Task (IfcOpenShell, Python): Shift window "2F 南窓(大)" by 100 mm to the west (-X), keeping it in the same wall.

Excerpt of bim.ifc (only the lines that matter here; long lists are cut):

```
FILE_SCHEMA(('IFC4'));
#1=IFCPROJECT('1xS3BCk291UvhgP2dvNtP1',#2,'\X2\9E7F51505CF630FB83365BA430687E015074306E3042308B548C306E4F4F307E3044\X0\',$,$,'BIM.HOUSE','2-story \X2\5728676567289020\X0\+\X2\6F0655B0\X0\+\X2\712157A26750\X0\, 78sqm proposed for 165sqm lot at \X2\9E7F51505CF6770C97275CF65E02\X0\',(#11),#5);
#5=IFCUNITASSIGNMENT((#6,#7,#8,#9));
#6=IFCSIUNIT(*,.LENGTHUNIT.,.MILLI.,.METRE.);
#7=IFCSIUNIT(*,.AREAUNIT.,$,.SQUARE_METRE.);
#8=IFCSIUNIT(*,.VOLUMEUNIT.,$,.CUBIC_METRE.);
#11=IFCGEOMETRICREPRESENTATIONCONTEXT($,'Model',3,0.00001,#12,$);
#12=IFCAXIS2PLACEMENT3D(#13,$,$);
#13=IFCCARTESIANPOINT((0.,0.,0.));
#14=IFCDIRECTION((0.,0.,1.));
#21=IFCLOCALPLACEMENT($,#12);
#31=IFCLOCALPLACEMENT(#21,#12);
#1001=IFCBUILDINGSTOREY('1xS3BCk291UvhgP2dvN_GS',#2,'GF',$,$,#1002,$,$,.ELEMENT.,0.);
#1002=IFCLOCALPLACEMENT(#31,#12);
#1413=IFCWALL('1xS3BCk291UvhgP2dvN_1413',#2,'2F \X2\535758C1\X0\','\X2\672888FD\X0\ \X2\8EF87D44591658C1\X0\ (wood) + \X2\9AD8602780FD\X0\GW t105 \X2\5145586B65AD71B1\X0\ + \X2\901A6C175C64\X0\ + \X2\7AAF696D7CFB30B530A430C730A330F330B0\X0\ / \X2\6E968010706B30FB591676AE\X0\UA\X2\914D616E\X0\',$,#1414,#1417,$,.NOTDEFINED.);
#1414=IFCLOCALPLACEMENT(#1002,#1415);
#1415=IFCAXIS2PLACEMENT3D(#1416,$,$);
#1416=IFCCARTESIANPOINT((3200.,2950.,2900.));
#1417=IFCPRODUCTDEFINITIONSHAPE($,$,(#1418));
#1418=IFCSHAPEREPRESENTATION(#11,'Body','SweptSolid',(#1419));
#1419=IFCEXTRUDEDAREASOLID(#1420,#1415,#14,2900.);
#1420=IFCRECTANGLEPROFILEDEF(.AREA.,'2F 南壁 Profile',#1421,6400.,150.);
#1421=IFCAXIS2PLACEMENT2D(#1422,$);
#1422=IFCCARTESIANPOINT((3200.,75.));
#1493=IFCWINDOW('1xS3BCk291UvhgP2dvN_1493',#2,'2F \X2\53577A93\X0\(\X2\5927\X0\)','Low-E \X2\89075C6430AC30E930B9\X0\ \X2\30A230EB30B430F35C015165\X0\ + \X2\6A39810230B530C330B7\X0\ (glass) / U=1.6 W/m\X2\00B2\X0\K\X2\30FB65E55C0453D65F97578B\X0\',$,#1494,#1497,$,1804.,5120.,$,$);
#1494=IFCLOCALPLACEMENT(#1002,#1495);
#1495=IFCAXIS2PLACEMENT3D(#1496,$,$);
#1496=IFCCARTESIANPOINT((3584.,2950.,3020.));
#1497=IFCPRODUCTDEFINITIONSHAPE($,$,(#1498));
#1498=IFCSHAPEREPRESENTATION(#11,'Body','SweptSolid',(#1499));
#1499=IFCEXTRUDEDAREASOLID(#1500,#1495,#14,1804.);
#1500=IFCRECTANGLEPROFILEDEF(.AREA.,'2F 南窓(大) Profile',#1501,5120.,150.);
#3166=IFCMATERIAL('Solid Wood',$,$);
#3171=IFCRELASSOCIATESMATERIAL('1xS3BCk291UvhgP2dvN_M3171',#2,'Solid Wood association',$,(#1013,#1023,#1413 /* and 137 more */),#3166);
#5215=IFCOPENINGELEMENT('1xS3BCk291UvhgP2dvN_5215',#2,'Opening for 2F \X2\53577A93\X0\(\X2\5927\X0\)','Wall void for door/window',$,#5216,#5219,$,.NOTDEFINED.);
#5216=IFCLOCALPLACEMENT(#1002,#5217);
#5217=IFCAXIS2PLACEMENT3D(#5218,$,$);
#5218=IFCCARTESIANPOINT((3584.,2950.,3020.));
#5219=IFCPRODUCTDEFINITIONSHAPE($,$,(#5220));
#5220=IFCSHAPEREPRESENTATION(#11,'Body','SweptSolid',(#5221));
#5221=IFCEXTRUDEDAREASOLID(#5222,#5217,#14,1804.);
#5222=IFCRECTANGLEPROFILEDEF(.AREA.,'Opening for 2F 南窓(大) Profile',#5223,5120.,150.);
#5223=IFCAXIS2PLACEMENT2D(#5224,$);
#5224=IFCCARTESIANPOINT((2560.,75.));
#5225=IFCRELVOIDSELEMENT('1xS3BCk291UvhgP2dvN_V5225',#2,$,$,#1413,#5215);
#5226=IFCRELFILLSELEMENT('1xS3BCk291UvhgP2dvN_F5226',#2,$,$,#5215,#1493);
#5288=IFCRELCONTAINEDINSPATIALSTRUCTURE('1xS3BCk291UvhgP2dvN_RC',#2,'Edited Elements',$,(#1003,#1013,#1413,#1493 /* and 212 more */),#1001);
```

```python
import ifcopenshell
import ifcopenshell.api.geometry
import ifcopenshell.util.placement
import ifcopenshell.util.unit

model = ifcopenshell.open("bim.ifc")
unit_scale = ifcopenshell.util.unit.calculate_unit_scale(model)

window = model.by_guid("1xS3BCk291UvhgP2dvN_1493")
opening = window.FillsVoids[0].RelatingOpeningElement
wall = opening.VoidsElements[0].RelatingBuildingElement

wall_matrix = ifcopenshell.util.placement.get_local_placement(wall.ObjectPlacement)
shift = wall_matrix[:3, 0] * -0.1 / unit_scale
before = ifcopenshell.util.placement.get_local_placement(window.ObjectPlacement)[:3, 3].copy()

# The window is not placed relative to its opening, so move both.
for product in (opening, window):
    matrix = ifcopenshell.util.placement.get_local_placement(product.ObjectPlacement)
    matrix[:3, 3] += shift
    ifcopenshell.api.geometry.edit_object_placement(model, product=product, matrix=matrix, is_si=False)

after = ifcopenshell.util.placement.get_local_placement(window.ObjectPlacement)[:3, 3]
print("window moved by", (after - before).round(3) + 0.0)

model.write("bim_rev.ifc")
```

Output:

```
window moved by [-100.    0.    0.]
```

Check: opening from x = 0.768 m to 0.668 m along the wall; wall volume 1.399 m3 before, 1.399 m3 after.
